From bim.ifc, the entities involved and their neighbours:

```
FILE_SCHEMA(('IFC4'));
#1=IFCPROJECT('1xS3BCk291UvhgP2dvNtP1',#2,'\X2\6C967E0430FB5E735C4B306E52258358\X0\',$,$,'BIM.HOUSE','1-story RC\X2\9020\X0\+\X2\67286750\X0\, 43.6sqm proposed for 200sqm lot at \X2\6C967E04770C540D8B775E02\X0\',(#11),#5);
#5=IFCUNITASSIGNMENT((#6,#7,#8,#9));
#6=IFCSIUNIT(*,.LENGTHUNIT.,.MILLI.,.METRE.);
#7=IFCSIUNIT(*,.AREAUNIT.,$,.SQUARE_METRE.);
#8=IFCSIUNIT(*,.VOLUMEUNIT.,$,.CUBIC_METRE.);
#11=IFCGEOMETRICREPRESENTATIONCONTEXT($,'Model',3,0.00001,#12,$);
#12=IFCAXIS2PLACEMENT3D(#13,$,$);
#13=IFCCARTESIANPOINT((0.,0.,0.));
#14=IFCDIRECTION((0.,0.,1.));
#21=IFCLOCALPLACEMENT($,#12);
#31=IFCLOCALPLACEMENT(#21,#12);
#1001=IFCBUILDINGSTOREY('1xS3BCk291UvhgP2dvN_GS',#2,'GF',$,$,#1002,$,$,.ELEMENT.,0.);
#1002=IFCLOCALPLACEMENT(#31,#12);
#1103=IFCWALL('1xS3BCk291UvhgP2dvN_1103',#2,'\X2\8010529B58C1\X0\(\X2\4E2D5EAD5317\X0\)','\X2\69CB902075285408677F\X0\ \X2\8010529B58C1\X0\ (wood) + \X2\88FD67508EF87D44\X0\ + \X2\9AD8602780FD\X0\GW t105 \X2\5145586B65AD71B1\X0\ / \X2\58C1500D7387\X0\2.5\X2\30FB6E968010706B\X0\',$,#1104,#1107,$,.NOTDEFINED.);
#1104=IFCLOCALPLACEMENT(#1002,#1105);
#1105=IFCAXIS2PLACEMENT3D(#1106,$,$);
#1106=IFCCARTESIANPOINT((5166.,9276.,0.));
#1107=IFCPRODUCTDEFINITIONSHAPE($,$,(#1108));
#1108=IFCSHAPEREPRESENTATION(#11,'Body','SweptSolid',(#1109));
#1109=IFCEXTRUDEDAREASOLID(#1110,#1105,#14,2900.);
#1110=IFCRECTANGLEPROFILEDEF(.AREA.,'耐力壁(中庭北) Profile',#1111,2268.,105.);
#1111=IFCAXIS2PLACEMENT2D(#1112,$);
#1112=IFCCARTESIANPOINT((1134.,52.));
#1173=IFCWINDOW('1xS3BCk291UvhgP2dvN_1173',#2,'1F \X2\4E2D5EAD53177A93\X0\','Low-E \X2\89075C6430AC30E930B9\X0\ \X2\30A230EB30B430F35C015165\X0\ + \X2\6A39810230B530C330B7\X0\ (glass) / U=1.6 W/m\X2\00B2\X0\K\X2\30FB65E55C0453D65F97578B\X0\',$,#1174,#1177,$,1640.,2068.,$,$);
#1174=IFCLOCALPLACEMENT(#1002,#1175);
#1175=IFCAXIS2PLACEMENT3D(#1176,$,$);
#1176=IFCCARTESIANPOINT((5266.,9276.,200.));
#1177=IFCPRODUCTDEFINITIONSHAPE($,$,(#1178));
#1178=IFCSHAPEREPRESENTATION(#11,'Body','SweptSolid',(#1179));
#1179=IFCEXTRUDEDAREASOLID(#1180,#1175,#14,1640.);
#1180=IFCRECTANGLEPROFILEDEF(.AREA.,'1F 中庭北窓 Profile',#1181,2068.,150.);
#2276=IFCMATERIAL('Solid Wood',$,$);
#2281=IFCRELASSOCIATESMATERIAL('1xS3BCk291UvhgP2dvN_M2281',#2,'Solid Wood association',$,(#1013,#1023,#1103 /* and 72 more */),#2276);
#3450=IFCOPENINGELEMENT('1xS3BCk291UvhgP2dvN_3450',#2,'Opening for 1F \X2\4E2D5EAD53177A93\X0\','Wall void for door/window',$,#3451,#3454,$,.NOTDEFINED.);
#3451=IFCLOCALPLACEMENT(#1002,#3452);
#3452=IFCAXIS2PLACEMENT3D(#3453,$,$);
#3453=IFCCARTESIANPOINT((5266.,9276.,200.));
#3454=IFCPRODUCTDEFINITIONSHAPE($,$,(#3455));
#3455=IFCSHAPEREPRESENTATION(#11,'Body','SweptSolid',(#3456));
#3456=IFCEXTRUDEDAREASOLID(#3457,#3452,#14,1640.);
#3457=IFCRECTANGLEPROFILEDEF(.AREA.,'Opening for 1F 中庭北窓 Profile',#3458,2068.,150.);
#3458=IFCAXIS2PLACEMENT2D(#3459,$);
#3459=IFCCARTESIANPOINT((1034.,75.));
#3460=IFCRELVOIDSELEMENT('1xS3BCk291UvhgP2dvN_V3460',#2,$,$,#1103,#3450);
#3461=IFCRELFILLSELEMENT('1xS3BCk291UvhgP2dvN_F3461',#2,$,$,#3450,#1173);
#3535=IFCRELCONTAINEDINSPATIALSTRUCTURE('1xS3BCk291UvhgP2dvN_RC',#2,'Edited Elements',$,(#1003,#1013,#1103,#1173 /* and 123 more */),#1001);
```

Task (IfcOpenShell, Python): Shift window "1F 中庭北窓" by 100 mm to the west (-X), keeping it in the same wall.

```python
import ifcopenshell
import ifcopenshell.api.geometry
import ifcopenshell.util.placement

model = ifcopenshell.open("bim.ifc")

window = model.by_guid("1xS3BCk291UvhgP2dvN_1173")
opening = window.FillsVoids[0].RelatingOpeningElement
wall = opening.VoidsElements[0].RelatingBuildingElement

wall_matrix = ifcopenshell.util.placement.get_local_placement(wall.ObjectPlacement)
shift = wall_matrix[:3, 0] * -100.0
before = ifcopenshell.util.placement.get_local_placement(window.ObjectPlacement)[:3, 3].copy()

# The window is not placed relative to its opening, so move both.
for product in (opening, window):
    matrix = ifcopenshell.util.placement.get_local_placement(product.ObjectPlacement)
    matrix[:3, 3] += shift
    ifcopenshell.api.geometry.edit_object_placement(model, product=product, matrix=matrix, is_si=False)

after = ifcopenshell.util.placement.get_local_placement(window.ObjectPlacement)[:3, 3]
print("window moved by", (after - before).round(3) + 0.0)

model.write("bim-out.ifc")
```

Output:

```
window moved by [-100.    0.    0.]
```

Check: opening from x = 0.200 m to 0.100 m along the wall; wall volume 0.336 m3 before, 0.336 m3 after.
